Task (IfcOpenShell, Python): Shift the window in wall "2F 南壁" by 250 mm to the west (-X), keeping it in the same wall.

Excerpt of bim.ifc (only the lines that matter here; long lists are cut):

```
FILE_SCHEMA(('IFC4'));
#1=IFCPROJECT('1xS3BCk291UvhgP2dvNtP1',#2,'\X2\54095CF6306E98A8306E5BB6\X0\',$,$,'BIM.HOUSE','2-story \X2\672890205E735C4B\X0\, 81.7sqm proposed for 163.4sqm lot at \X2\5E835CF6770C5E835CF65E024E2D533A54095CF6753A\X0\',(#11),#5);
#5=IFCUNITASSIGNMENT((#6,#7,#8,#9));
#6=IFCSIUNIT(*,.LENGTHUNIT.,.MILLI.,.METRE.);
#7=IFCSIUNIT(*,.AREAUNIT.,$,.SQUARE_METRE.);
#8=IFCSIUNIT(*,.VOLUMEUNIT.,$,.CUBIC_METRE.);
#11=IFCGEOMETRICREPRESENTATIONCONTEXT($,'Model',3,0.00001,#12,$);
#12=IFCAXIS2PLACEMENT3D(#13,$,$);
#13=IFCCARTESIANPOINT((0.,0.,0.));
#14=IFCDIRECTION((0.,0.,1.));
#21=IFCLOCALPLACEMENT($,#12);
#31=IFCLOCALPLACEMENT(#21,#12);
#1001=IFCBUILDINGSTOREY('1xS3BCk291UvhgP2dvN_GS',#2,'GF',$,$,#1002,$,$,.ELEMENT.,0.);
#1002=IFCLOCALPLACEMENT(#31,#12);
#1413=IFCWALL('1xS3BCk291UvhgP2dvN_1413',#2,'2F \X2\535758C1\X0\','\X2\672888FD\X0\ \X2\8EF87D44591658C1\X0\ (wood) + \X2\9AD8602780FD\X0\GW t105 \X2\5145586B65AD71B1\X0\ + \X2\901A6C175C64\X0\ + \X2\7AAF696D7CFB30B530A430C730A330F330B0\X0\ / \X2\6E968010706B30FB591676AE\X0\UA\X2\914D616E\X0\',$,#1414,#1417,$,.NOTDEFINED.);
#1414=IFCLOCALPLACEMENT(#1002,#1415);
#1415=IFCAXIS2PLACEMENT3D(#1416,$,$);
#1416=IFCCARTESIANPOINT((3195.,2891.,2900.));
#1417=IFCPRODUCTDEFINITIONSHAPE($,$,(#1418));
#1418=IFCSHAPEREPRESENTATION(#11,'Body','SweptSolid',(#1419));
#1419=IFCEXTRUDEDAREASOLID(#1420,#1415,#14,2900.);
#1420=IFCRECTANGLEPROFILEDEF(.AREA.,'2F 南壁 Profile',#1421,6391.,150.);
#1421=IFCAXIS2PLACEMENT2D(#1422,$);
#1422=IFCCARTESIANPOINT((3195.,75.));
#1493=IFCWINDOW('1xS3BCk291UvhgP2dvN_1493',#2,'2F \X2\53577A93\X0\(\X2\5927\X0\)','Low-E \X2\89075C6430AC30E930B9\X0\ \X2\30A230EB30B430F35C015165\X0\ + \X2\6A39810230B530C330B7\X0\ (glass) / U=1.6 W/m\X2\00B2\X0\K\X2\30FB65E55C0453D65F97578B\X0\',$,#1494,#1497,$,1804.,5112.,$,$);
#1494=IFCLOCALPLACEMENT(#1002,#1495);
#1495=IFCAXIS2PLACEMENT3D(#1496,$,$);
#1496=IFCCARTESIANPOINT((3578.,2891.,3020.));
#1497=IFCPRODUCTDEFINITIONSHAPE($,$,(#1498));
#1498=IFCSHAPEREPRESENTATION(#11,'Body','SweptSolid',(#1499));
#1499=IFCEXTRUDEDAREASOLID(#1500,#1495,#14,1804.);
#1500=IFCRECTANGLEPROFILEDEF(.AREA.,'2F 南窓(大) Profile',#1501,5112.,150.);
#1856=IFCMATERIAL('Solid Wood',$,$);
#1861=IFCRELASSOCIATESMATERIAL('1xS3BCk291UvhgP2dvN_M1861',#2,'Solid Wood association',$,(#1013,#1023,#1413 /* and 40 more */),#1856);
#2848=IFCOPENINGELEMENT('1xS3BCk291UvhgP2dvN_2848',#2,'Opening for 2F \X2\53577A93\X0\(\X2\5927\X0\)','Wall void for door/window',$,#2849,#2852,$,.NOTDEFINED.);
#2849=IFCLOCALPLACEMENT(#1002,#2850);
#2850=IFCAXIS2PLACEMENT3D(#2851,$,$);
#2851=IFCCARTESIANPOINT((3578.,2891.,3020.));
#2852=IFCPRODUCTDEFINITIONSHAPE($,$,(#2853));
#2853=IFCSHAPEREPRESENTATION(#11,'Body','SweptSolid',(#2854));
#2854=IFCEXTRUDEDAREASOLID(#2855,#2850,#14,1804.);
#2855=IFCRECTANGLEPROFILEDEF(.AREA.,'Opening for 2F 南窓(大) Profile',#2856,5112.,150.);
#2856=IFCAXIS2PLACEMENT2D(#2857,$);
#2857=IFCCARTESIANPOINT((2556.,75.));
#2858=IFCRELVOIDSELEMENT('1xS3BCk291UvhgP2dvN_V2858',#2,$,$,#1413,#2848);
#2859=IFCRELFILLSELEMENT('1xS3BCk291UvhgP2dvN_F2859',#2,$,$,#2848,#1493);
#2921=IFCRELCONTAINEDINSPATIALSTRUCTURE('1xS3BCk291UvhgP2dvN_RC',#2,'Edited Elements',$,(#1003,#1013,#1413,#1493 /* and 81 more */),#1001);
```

```python
import ifcopenshell
import ifcopenshell.api.geometry
import ifcopenshell.util.placement

model = ifcopenshell.open("bim.ifc")

window = model.by_id(1493)
opening = window.FillsVoids[0].RelatingOpeningElement
wall = opening.VoidsElements[0].RelatingBuildingElement

wall_matrix = ifcopenshell.util.placement.get_local_placement(wall.ObjectPlacement)
shift = wall_matrix[:3, 0] * -250.0
before = ifcopenshell.util.placement.get_local_placement(window.ObjectPlacement)[:3, 3].copy()

# The window is not placed relative to its opening, so move both.
for product in (opening, window):
    matrix = ifcopenshell.util.placement.get_local_placement(product.ObjectPlacement)
    matrix[:3, 3] += shift
    ifcopenshell.api.geometry.edit_object_placement(model, product=product, matrix=matrix, is_si=False)

after = ifcopenshell.util.placement.get_local_placement(window.ObjectPlacement)[:3, 3]
print("window moved by", (after - before).round(3) + 0.0)

model.write("bim_updated.ifc")
```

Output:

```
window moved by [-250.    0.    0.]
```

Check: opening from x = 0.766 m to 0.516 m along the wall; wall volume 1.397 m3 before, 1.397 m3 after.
